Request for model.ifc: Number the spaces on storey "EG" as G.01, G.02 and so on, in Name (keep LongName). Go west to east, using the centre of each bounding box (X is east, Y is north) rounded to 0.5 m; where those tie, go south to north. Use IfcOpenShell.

First a look at what the model holds.

```python
import ifcopenshell
import ifcopenshell.util.element
import ifcopenshell.util.placement

model = ifcopenshell.open("model.ifc")
print(model.schema)
storey = next(s for s in model.by_type("IfcBuildingStorey") if s.Name == "EG")
spaces = [e for e in ifcopenshell.util.element.get_decomposition(storey) if e.is_a("IfcSpace")]
for e in sorted(spaces, key=lambda e: e.id()):
    origin = ifcopenshell.util.placement.get_local_placement(e.ObjectPlacement)[:3, 3]
    print(e.id(), e.Name, e.LongName, origin.round(2) + 0.0, sep=" | ")
```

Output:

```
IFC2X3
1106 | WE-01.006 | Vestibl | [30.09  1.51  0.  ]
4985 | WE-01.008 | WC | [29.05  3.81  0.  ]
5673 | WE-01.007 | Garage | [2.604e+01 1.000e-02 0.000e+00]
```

```python
import ifcopenshell
import ifcopenshell.geom
import ifcopenshell.util.element
import ifcopenshell.util.shape

model = ifcopenshell.open("model.ifc")
settings = ifcopenshell.geom.settings()
settings.set("use-world-coords", True)


def centre(element):
    shape = ifcopenshell.geom.create_shape(settings, element)
    return ifcopenshell.util.shape.get_bbox_centroid(shape.geometry)


storey = next(s for s in model.by_type("IfcBuildingStorey") if s.Name == "EG")
spaces = [e for e in ifcopenshell.util.element.get_decomposition(storey) if e.is_a("IfcSpace")]

# Insertion points can sit at a corner or the storey origin, so sort by the geometry (in metres).
centres = {e: centre(e) for e in spaces}
spaces.sort(key=lambda e: (round(centres[e][0] / 0.5), centres[e][1]))

for i, e in enumerate(spaces, start=1):
    number = f"G.{i:02d}"
    e.Name = number
    print(e.id(), number)

model.write("model_v2.ifc")
```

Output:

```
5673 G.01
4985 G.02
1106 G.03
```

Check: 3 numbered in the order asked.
